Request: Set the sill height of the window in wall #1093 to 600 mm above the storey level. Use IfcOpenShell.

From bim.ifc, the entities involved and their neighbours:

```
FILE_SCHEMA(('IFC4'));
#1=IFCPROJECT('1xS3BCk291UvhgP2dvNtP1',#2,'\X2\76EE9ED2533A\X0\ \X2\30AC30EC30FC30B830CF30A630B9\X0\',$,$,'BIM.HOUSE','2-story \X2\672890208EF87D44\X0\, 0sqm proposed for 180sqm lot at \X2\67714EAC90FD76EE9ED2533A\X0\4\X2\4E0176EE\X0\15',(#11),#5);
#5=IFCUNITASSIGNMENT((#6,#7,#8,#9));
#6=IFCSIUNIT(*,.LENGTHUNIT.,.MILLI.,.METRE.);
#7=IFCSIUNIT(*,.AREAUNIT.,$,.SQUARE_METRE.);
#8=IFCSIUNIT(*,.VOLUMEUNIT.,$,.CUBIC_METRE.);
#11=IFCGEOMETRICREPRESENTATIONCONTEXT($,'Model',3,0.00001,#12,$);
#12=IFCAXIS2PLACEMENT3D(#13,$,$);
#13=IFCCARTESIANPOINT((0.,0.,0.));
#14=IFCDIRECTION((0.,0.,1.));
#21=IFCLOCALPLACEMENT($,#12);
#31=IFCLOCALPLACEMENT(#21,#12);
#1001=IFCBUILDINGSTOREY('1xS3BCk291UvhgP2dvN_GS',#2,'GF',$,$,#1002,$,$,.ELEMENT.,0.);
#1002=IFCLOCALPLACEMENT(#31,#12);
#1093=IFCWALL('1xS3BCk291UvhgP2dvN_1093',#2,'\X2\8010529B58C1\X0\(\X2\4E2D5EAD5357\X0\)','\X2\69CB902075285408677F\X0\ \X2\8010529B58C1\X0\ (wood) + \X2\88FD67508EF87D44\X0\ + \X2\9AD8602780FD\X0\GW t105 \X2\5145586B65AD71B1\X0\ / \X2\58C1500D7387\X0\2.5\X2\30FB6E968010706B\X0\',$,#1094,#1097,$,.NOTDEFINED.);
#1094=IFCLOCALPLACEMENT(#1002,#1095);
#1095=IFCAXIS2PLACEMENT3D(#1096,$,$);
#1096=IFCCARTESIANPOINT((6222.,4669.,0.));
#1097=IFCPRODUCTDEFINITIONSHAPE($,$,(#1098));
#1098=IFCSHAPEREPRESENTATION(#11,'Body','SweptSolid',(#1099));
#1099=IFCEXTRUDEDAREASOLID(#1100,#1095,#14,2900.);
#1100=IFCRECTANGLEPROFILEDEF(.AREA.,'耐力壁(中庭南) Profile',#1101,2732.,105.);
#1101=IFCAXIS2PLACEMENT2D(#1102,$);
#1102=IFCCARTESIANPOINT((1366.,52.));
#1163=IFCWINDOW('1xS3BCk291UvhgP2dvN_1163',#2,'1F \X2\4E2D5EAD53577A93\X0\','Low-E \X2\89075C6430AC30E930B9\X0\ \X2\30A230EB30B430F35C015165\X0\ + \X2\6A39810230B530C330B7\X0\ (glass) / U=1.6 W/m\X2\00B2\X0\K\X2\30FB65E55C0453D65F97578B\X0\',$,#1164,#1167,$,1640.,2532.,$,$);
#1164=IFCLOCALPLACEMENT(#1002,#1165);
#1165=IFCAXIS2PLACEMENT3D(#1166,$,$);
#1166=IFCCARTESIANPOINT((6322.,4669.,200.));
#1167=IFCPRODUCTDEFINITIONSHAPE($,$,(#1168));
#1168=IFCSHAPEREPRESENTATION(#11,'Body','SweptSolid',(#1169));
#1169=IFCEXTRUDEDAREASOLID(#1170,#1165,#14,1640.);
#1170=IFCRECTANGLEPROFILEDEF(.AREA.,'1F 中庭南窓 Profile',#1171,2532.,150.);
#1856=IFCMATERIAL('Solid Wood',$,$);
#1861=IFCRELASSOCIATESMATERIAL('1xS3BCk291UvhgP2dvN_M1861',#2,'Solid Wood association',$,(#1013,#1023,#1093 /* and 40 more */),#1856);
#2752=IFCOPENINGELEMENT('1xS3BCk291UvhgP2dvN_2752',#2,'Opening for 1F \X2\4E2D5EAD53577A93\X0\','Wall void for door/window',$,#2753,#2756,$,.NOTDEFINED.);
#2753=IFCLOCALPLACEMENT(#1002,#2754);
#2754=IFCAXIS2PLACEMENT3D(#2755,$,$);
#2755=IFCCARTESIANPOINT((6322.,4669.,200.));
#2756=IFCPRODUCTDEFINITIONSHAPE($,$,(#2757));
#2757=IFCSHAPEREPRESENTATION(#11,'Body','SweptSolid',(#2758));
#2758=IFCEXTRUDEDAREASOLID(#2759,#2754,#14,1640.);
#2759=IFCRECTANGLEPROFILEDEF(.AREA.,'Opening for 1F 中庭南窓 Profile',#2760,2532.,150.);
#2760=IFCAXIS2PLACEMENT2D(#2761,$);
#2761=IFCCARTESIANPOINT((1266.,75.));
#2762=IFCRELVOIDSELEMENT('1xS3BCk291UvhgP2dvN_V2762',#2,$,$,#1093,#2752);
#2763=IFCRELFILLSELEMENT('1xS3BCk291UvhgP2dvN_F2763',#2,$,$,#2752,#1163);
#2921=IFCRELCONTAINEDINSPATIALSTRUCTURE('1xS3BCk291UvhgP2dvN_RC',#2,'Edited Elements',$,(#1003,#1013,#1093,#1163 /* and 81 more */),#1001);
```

```python
import numpy as np
import ifcopenshell
import ifcopenshell.api.geometry
import ifcopenshell.geom
import ifcopenshell.util.element
import ifcopenshell.util.placement
import ifcopenshell.util.shape
import ifcopenshell.util.unit

model = ifcopenshell.open("bim.ifc")
unit_scale = ifcopenshell.util.unit.calculate_unit_scale(model)

window = model.by_id(1163)
opening = window.FillsVoids[0].RelatingOpeningElement
storey = ifcopenshell.util.element.get_container(window, ifc_class="IfcBuildingStorey")
level = ifcopenshell.util.placement.get_local_placement(storey.ObjectPlacement)[2, 3]

# The opening's origin need not be at the sill, so measure its lowest point.
shape = ifcopenshell.geom.create_shape(ifcopenshell.geom.settings(), opening)
bottom = ifcopenshell.util.shape.get_shape_bottom_elevation(shape, shape.geometry) / unit_scale
dz = level + 0.6 / unit_scale - bottom

shift = np.array([0.0, 0.0, dz])
# The window is not placed relative to its opening, so move both.
for product in (opening, window):
    matrix = ifcopenshell.util.placement.get_local_placement(product.ObjectPlacement)
    matrix[:3, 3] += shift
    ifcopenshell.api.geometry.edit_object_placement(model, product=product, matrix=matrix, is_si=False)

print(f"moved by {dz * unit_scale:+.3f} m")

model.write("bim_edited.ifc")
```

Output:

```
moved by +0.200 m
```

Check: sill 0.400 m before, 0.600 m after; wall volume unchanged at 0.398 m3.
